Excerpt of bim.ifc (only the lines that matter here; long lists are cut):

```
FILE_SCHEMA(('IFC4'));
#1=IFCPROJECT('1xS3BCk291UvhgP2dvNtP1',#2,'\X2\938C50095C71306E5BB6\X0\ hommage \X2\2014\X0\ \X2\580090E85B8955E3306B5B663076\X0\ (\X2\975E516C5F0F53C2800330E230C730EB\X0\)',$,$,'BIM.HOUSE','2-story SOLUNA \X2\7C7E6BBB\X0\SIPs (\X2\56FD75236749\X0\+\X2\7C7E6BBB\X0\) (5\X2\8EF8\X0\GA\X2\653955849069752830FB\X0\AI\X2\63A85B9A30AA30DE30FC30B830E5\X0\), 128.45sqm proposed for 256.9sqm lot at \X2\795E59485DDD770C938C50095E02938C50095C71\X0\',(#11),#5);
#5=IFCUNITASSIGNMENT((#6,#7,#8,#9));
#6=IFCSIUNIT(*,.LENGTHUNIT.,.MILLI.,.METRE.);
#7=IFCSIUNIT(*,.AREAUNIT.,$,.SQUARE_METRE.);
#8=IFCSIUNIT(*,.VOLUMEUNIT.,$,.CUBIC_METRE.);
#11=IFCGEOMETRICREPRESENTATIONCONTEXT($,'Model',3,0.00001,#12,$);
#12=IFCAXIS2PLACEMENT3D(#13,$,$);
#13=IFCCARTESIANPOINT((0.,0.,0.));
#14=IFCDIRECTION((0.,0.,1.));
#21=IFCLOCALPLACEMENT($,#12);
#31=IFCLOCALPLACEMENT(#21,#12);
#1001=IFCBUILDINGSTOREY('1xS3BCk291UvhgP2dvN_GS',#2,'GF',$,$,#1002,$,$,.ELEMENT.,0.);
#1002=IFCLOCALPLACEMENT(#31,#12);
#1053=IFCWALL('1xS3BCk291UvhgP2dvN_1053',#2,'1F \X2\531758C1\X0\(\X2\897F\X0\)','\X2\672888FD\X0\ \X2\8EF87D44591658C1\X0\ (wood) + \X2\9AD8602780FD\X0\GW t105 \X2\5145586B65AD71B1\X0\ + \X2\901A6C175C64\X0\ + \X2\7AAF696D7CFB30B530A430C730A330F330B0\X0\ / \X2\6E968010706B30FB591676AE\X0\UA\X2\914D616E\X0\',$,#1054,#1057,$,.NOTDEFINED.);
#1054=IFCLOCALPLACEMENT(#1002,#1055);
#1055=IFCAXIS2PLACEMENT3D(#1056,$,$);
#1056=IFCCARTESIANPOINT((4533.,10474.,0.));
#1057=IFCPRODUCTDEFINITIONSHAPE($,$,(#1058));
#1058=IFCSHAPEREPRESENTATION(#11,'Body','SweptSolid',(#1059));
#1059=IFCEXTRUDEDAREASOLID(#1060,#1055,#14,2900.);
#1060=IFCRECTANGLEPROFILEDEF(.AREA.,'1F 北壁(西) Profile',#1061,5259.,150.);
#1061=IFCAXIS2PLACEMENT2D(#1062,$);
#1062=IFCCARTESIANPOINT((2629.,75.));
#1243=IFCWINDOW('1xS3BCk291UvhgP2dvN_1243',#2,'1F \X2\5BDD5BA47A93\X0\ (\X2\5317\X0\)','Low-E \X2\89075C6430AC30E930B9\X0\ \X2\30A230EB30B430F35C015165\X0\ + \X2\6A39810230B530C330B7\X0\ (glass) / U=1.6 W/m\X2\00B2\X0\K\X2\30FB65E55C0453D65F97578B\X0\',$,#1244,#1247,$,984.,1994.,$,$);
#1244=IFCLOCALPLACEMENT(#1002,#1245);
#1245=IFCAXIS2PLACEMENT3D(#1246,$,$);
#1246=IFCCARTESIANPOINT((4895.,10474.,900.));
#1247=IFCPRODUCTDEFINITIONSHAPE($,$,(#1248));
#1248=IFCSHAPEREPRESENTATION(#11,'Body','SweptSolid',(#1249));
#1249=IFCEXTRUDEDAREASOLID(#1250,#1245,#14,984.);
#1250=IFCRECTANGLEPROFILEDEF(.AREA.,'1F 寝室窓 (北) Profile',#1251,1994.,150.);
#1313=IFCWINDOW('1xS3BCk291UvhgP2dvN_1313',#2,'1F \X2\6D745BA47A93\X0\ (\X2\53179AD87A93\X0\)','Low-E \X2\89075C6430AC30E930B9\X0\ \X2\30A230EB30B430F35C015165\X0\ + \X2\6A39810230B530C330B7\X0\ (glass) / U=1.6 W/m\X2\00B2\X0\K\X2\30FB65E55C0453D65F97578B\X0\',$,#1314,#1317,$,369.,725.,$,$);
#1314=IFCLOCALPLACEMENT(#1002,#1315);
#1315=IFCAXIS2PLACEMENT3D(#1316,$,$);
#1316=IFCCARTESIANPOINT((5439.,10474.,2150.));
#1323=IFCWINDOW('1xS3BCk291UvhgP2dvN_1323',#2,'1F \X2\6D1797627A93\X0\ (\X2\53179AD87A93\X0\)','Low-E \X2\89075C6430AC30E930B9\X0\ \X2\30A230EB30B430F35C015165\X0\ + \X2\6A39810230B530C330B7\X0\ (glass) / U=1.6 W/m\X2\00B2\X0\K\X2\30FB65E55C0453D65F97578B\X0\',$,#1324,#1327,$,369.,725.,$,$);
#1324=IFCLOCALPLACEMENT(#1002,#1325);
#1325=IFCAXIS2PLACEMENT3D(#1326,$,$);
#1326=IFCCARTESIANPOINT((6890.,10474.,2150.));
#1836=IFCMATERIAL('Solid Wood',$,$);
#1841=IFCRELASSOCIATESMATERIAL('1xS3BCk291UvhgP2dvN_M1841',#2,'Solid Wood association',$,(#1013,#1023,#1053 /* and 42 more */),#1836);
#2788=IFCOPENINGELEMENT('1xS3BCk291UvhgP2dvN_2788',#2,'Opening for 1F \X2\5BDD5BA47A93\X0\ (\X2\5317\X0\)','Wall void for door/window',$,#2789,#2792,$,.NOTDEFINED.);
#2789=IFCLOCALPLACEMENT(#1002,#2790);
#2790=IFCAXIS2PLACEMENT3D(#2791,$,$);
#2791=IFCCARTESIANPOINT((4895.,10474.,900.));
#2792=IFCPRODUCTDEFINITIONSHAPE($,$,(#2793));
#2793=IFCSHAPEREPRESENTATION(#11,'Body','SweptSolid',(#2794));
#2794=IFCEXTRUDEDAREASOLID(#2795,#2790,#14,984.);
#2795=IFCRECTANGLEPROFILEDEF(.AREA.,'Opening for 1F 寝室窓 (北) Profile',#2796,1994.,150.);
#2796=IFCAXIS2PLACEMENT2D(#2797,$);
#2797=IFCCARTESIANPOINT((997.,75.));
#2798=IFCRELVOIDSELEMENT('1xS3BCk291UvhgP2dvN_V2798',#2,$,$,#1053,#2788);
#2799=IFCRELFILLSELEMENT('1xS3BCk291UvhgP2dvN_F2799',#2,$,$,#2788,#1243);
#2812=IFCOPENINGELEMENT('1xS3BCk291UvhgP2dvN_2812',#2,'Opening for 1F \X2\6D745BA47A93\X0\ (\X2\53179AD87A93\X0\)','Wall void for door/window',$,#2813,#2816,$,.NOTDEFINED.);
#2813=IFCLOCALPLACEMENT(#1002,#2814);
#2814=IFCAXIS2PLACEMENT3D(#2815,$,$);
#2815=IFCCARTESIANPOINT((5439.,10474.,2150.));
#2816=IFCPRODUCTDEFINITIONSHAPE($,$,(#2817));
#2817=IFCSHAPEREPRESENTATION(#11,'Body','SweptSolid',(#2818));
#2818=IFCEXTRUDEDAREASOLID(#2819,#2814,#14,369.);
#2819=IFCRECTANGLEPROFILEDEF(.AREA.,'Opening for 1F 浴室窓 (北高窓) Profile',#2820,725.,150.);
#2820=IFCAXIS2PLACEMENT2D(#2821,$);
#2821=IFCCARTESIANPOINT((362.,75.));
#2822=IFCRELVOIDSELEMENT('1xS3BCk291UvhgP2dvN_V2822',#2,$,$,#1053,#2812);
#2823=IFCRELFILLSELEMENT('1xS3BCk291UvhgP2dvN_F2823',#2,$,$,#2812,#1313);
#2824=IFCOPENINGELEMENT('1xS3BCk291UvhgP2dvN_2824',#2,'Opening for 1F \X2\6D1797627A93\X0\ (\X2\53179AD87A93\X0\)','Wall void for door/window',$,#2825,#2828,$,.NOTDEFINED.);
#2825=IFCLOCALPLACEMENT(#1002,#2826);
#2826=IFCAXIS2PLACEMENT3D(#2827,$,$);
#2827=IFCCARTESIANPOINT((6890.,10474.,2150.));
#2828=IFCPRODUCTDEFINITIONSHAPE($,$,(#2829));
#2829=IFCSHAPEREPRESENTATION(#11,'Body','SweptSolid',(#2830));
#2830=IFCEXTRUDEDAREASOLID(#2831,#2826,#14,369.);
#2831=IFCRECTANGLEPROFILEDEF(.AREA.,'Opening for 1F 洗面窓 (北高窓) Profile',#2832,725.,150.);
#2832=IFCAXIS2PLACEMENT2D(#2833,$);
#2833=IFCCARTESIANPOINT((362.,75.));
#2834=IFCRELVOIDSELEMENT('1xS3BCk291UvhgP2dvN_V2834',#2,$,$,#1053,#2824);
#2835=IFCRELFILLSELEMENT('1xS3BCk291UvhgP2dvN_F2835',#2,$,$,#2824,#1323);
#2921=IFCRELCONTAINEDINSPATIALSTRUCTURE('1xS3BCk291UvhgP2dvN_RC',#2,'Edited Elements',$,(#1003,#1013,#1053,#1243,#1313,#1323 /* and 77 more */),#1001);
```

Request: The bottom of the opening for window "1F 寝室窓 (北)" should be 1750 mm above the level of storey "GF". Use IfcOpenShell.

```python
import numpy as np
import ifcopenshell
import ifcopenshell.api.geometry
import ifcopenshell.geom
import ifcopenshell.util.element
import ifcopenshell.util.placement
import ifcopenshell.util.shape
import ifcopenshell.util.unit

model = ifcopenshell.open("bim.ifc")
unit_scale = ifcopenshell.util.unit.calculate_unit_scale(model)

window = model.by_guid("1xS3BCk291UvhgP2dvN_1243")
opening = window.FillsVoids[0].RelatingOpeningElement
storey = ifcopenshell.util.element.get_container(window, ifc_class="IfcBuildingStorey")
level = ifcopenshell.util.placement.get_local_placement(storey.ObjectPlacement)[2, 3]

# The opening's origin need not be at the sill, so measure its lowest point.
shape = ifcopenshell.geom.create_shape(ifcopenshell.geom.settings(), opening)
bottom = ifcopenshell.util.shape.get_shape_bottom_elevation(shape, shape.geometry) / unit_scale
dz = level + 1750.0 - bottom

shift = np.array([0.0, 0.0, dz])
# The window is not placed relative to its opening, so move both.
for product in (opening, window):
    matrix = ifcopenshell.util.placement.get_local_placement(product.ObjectPlacement)
    matrix[:3, 3] += shift
    ifcopenshell.api.geometry.edit_object_placement(model, product=product, matrix=matrix, is_si=False)

print(f"moved by {dz * unit_scale:+.3f} m")

model.write("bim_v2.ifc")
```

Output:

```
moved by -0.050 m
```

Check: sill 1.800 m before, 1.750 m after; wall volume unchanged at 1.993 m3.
